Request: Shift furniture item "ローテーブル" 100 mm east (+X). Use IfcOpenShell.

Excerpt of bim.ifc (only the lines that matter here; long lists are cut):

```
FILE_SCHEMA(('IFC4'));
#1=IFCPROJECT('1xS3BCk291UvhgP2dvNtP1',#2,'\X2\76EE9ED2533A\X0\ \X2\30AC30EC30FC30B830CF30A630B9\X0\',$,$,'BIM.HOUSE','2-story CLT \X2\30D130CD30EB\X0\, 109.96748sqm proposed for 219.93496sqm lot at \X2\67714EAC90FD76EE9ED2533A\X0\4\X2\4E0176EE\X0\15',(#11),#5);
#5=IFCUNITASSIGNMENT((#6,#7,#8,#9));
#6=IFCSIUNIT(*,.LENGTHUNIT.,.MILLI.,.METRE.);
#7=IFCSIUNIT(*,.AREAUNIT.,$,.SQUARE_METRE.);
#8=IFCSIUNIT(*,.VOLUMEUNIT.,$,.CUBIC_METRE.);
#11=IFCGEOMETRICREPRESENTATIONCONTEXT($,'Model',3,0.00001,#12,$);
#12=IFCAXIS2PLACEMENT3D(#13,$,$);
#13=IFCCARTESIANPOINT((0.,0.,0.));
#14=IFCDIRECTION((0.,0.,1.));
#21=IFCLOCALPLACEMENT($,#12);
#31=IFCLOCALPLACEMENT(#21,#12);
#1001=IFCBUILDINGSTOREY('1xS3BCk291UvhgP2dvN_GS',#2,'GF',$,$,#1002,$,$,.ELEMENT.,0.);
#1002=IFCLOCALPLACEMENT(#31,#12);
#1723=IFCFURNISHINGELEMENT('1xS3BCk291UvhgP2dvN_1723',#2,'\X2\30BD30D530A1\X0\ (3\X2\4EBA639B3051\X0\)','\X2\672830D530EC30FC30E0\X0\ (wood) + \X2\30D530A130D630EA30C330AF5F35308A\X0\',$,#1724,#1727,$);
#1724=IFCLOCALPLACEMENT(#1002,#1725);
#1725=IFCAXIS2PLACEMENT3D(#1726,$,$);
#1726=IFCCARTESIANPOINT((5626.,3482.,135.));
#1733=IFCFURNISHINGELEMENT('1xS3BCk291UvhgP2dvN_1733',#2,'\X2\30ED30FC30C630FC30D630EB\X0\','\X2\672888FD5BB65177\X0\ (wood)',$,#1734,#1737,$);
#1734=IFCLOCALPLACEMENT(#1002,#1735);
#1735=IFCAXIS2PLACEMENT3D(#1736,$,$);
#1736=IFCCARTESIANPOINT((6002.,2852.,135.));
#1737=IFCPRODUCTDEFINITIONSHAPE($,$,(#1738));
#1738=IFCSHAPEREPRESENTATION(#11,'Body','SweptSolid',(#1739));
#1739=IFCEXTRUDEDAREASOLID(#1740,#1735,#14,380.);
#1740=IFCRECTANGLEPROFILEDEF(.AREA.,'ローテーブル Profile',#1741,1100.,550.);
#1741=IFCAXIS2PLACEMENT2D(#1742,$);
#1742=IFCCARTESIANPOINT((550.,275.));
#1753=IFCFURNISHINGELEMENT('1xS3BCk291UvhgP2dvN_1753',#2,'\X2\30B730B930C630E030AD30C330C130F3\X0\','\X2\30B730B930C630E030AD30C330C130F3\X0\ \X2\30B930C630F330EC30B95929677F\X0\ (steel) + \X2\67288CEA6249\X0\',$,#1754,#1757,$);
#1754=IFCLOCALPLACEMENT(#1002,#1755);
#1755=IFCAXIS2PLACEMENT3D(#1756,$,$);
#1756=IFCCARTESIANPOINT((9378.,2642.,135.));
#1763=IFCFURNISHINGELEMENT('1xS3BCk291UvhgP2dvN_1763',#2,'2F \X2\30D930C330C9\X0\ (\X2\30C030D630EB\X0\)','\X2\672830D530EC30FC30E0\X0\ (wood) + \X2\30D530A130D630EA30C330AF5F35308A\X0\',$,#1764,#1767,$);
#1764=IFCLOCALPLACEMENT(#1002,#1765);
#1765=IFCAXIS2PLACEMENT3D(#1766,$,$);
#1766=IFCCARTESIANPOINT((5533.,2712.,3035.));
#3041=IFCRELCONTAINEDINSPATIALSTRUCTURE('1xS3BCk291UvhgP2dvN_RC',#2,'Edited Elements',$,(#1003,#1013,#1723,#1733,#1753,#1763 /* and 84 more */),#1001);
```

```python
import ifcopenshell
import ifcopenshell.api.geometry
import ifcopenshell.util.placement
import ifcopenshell.util.unit

model = ifcopenshell.open("bim.ifc")
unit_scale = ifcopenshell.util.unit.calculate_unit_scale(model)

item = model.by_guid("1xS3BCk291UvhgP2dvN_1733")
matrix = ifcopenshell.util.placement.get_local_placement(item.ObjectPlacement)
matrix[0, 3] += 0.1 / unit_scale
ifcopenshell.api.geometry.edit_object_placement(model, product=item, matrix=matrix, is_si=False)

print(ifcopenshell.util.placement.get_local_placement(item.ObjectPlacement).round(3) + 0.0)

model.write("bim_edited.ifc")
```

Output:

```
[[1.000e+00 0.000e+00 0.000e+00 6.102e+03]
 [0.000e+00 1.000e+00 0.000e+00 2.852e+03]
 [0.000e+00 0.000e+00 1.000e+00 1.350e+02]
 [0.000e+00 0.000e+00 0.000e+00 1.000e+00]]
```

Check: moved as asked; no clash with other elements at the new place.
